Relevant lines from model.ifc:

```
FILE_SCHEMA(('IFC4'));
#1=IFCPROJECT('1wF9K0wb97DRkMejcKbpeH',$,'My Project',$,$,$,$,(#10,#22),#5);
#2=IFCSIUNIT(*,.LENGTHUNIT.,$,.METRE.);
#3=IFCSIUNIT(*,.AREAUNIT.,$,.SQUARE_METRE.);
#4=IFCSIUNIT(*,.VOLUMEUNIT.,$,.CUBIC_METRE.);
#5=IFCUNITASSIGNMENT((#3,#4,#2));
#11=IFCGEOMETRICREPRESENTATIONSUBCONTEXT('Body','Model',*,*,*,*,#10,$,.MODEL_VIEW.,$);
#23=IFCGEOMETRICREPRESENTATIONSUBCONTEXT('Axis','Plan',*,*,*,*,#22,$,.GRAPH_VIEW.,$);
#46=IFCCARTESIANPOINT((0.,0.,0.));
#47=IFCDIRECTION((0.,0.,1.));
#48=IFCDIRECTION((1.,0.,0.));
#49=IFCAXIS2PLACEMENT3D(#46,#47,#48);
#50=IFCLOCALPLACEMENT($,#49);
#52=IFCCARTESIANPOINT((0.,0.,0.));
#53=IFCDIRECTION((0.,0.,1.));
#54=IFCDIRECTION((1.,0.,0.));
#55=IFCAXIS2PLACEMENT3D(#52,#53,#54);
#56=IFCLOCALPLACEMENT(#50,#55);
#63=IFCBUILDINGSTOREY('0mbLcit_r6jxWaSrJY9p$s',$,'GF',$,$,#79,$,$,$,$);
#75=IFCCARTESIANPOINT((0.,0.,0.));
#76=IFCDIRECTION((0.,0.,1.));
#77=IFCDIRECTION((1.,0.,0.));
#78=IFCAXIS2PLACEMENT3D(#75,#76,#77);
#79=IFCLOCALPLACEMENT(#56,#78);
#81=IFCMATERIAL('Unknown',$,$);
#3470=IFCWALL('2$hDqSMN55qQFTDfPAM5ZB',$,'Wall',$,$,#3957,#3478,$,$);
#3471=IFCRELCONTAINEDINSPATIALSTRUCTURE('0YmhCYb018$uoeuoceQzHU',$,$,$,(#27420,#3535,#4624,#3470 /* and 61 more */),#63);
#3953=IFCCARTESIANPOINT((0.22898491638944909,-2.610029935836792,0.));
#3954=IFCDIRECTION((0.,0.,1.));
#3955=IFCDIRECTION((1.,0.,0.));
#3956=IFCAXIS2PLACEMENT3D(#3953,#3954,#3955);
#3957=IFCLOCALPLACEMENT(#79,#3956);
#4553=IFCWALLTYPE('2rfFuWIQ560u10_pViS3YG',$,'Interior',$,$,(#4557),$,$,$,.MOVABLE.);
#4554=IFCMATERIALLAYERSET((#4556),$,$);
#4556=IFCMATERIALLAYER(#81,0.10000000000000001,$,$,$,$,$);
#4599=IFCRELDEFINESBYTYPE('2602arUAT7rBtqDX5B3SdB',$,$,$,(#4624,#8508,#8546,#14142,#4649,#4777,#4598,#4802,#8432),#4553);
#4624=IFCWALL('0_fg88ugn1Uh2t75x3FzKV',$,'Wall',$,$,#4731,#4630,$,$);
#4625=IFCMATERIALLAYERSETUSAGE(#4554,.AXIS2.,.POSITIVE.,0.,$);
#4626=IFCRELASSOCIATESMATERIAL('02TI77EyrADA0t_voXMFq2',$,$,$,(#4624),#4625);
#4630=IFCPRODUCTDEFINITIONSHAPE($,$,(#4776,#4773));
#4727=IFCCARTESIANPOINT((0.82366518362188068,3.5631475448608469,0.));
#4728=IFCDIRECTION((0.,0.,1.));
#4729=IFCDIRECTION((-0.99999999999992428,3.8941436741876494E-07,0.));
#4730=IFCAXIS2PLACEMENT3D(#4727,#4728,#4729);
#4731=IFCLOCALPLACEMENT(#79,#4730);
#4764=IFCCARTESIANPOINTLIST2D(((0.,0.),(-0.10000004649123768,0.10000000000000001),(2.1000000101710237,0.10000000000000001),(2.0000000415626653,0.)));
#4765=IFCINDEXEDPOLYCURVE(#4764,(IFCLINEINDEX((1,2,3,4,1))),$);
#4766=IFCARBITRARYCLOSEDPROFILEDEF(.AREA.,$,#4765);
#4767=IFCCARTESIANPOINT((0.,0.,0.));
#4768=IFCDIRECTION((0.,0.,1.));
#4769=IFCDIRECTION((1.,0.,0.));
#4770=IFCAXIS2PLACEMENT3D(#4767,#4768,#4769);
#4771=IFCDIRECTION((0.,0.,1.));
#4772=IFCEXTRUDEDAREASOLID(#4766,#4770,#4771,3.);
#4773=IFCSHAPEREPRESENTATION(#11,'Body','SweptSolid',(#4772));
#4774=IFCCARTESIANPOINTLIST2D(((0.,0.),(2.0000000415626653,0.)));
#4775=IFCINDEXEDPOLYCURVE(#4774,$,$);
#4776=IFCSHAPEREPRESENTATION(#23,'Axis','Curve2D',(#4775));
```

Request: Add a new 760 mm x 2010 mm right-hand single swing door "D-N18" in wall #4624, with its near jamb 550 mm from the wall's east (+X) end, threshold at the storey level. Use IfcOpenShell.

```python
import numpy as np
import ifcopenshell
import ifcopenshell.api.feature
import ifcopenshell.api.geometry
import ifcopenshell.api.root
import ifcopenshell.api.spatial
import ifcopenshell.geom
import ifcopenshell.util.element
import ifcopenshell.util.placement
import ifcopenshell.util.representation
import ifcopenshell.util.shape
import ifcopenshell.util.unit

model = ifcopenshell.open("model.ifc")
unit_scale = ifcopenshell.util.unit.calculate_unit_scale(model)
settings = ifcopenshell.geom.settings()


def volume(element):
    """Net volume in cubic metres, openings subtracted."""
    shape = ifcopenshell.geom.create_shape(settings, element)
    return ifcopenshell.util.shape.get_volume(shape.geometry)


wall = model.by_guid("0_fg88ugn1Uh2t75x3FzKV")
storey = ifcopenshell.util.element.get_container(wall, ifc_class="IfcBuildingStorey")
context = ifcopenshell.util.representation.get_context(model, "Model", "Body", "MODEL_VIEW")
before = volume(wall)

width, height, from_end, sill = 0.76, 2.01, 0.55, 0.0  # metres

# The wall runs along its own X axis, and the end named is its -X end.
wall_shape = ifcopenshell.geom.create_shape(settings, wall)
x, y, z = ifcopenshell.util.shape.get_vertices(wall_shape.geometry).T
start = x.min() + from_end
face, thickness = float(y.min()), float(y.max() - y.min())
wall_matrix = ifcopenshell.util.placement.get_local_placement(wall.ObjectPlacement)
level = ifcopenshell.util.placement.get_local_placement(storey.ObjectPlacement)[2, 3]


def in_wall(x, y):
    """Placement at x, y metres in the wall's axes, at sill height."""
    matrix = wall_matrix.copy()
    matrix[:, 3] = wall_matrix @ np.array([x / unit_scale, y / unit_scale, 0.0, 1.0])
    matrix[2, 3] = level + sill / unit_scale
    return matrix


# Opening: a box that overshoots both wall faces by 50 mm.
opening = ifcopenshell.api.root.create_entity(model, ifc_class="IfcOpeningElement", predefined_type="OPENING")
box = ifcopenshell.api.geometry.add_wall_representation(
    model, context=context, length=width, height=height, thickness=thickness + 0.1
)
ifcopenshell.api.geometry.assign_representation(model, product=opening, representation=box)
ifcopenshell.api.geometry.edit_object_placement(model, product=opening, matrix=in_wall(start, face - 0.05), is_si=False)
ifcopenshell.api.feature.add_feature(model, feature=opening, element=wall)

door = ifcopenshell.api.root.create_entity(model, ifc_class="IfcDoor", name="D-N18", predefined_type="DOOR")
door.OverallWidth, door.OverallHeight = width / unit_scale, height / unit_scale
door.OperationType = "SINGLE_SWING_RIGHT"
body = ifcopenshell.api.geometry.add_door_representation(
    model,
    context=context,
    overall_width=door.OverallWidth,
    overall_height=door.OverallHeight,
    operation_type="SINGLE_SWING_RIGHT",
    lining_properties={"LiningDepth": thickness / unit_scale, "ThresholdDepth": thickness / unit_scale},
)
ifcopenshell.api.geometry.assign_representation(model, product=door, representation=body)
ifcopenshell.api.spatial.assign_container(model, products=[door], relating_structure=storey)
ifcopenshell.api.feature.add_filling(model, opening=opening, element=door)

# The lining spans the wall, so the door starts at the wall face.
ifcopenshell.api.geometry.edit_object_placement(model, product=door, matrix=in_wall(start, face), is_si=False)

after = volume(wall)

print(f"wall volume {before:.3f} -> {after:.3f} m3")

model.write("model_updated.ifc")
```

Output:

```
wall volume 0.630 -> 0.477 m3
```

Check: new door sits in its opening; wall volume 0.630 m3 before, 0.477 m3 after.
